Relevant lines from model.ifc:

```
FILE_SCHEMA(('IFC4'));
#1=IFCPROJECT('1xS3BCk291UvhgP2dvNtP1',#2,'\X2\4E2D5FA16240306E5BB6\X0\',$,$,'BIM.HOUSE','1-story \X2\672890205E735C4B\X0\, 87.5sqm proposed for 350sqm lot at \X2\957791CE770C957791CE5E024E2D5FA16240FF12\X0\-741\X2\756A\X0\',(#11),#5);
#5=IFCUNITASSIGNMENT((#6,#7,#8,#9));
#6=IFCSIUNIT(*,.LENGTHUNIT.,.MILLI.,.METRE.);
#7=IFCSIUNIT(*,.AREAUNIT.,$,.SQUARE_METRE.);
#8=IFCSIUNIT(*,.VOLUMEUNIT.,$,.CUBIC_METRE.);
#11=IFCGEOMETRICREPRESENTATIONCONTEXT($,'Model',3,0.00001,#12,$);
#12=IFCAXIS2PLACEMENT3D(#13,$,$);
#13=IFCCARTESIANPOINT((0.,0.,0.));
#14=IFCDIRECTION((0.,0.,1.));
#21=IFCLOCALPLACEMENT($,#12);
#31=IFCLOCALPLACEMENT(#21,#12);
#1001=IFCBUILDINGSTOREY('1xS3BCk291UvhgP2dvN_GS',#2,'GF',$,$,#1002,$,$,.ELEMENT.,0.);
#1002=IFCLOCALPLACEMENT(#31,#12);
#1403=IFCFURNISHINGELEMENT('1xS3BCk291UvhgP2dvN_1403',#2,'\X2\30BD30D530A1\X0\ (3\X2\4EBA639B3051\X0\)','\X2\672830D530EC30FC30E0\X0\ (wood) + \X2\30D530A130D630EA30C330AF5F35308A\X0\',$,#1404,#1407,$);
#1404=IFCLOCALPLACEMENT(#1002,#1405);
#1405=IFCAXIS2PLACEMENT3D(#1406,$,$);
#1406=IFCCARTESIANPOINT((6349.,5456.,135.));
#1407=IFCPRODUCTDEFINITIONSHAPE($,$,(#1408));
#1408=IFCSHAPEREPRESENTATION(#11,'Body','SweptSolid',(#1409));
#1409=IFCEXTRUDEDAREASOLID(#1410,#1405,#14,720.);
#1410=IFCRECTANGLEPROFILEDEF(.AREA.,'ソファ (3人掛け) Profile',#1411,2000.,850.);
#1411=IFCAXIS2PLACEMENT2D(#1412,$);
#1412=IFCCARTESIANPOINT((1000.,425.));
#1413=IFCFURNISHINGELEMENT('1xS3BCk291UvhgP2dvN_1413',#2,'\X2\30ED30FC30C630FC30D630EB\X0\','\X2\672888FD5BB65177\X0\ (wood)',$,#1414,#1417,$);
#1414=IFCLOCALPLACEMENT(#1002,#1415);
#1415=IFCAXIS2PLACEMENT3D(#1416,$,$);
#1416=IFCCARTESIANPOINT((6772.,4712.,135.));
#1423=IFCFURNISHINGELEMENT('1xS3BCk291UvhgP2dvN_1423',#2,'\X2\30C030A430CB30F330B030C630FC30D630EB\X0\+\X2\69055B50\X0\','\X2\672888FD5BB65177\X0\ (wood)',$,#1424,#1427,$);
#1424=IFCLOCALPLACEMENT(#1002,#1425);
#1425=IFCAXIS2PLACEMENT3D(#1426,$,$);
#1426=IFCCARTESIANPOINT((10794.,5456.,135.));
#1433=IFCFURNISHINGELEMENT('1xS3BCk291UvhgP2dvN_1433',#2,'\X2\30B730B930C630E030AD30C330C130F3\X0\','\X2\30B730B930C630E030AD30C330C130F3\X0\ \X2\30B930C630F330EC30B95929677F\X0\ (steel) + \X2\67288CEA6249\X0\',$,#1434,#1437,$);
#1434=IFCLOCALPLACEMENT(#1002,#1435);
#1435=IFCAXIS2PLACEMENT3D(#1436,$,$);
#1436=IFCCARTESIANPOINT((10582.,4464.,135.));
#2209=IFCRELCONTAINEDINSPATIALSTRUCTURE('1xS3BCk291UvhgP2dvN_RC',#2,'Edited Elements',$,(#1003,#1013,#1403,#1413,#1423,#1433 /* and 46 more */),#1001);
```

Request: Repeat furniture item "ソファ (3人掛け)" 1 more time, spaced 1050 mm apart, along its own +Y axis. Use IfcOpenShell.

```python
import ifcopenshell
import ifcopenshell.api.geometry
import ifcopenshell.api.root
import ifcopenshell.util.element
import ifcopenshell.util.placement

model = ifcopenshell.open("model.ifc")


def reuse_history(source, copy):
    """copy_class also copies each property set's owner history, people and application; keep the originals."""
    for rel in copy.IsDefinedBy:
        if rel.is_a("IfcRelDefinesByProperties") and (history := rel.RelatingPropertyDefinition.OwnerHistory):
            rel.RelatingPropertyDefinition.OwnerHistory = source.OwnerHistory
            ifcopenshell.util.element.remove_deep2(model, history)


source = model.by_guid("1xS3BCk291UvhgP2dvN_1403")
base = ifcopenshell.util.placement.get_local_placement(source.ObjectPlacement)
step = base[:3, 1] * 1050.0

for i in range(1, 2):
    copy = ifcopenshell.api.root.copy_class(model, product=source)
    copy.Representation = ifcopenshell.util.element.copy_deep(
        model, source.Representation, exclude=["IfcGeometricRepresentationContext", "IfcRepresentationMap"]
    )
    reuse_history(source, copy)
    matrix = base.copy()
    matrix[:3, 3] += i * step
    print("added at", matrix[:3, 3].round(3) + 0.0)
    ifcopenshell.api.geometry.edit_object_placement(model, product=copy, matrix=matrix, is_si=False)

model.write("model_edited.ifc")
```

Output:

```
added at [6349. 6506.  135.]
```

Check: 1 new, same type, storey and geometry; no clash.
